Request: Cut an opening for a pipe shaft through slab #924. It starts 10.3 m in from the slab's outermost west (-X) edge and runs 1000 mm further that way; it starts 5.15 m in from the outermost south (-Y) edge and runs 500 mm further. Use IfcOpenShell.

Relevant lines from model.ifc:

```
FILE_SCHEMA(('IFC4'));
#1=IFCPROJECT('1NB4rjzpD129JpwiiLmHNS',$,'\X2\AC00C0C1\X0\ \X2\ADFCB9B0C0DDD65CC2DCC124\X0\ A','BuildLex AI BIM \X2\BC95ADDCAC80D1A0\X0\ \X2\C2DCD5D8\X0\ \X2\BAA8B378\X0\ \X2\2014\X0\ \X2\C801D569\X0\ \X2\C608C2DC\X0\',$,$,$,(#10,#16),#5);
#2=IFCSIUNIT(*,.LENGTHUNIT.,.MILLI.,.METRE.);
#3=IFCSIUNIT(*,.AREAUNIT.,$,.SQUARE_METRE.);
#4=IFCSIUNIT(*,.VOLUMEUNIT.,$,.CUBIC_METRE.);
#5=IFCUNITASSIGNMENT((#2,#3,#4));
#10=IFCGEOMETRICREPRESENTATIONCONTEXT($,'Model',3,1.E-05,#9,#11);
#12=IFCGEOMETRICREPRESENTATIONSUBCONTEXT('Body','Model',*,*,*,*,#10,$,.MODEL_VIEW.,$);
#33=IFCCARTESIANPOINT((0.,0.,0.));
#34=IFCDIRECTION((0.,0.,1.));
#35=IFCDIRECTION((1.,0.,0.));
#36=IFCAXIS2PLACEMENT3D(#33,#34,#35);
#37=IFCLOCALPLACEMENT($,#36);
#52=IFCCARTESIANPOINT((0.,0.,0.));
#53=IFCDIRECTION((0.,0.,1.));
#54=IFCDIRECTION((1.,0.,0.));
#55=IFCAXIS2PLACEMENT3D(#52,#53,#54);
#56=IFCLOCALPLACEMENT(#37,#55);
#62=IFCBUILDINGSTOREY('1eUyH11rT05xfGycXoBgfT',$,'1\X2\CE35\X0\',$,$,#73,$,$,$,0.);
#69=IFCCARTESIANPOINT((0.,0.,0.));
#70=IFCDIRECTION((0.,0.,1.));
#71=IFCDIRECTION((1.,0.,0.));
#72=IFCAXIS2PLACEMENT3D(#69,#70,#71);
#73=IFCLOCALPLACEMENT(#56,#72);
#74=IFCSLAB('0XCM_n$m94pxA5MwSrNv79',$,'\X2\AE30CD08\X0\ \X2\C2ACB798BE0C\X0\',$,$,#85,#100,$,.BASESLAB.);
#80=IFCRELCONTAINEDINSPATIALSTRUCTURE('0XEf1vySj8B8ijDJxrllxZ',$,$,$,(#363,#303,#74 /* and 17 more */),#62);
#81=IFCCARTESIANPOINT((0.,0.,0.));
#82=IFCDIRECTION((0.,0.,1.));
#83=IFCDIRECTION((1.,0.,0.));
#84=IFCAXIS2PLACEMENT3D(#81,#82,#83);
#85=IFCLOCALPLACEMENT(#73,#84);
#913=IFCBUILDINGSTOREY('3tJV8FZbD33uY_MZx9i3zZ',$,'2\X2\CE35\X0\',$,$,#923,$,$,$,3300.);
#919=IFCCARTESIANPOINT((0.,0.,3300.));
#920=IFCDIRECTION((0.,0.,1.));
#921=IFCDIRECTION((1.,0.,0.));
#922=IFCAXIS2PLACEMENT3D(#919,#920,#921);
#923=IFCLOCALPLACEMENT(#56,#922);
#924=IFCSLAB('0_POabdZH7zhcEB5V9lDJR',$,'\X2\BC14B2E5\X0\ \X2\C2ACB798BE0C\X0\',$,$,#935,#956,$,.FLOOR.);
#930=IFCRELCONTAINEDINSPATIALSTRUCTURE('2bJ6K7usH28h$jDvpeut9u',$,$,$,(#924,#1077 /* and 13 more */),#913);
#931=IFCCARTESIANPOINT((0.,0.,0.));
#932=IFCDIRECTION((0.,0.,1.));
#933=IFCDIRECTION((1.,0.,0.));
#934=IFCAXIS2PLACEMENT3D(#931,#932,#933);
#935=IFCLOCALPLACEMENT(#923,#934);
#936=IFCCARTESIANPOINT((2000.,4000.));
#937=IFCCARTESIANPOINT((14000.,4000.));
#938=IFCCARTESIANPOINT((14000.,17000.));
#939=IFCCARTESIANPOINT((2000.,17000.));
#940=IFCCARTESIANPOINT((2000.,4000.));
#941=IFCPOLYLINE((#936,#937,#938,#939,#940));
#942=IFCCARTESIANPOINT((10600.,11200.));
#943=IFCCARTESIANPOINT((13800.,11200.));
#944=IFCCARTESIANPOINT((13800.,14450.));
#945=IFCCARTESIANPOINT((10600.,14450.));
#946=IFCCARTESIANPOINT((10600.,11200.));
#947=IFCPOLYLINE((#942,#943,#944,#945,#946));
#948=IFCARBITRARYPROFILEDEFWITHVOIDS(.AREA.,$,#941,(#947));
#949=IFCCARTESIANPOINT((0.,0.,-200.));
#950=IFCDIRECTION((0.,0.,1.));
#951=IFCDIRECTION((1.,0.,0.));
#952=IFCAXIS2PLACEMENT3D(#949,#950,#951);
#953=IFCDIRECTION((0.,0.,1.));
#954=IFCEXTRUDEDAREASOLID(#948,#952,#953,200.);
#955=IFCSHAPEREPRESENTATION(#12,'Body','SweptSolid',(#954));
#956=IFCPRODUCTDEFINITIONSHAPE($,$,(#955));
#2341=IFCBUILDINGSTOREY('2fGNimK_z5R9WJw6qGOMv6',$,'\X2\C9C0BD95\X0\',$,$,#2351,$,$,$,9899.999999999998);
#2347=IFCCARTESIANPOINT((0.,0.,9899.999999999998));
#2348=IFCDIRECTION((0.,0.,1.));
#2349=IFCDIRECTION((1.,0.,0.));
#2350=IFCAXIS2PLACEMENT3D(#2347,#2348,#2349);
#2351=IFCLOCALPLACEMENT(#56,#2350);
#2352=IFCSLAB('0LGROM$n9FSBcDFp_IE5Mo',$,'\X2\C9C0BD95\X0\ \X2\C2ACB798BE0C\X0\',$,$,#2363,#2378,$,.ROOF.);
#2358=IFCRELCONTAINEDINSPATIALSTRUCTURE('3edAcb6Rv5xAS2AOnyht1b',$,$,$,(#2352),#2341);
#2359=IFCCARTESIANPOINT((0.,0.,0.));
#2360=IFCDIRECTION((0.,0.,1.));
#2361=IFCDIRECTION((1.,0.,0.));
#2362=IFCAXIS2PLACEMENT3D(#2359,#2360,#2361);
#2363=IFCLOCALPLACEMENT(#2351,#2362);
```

```python
import numpy as np
import ifcopenshell
import ifcopenshell.api.feature
import ifcopenshell.api.geometry
import ifcopenshell.api.root
import ifcopenshell.geom
import ifcopenshell.util.placement
import ifcopenshell.util.representation
import ifcopenshell.util.shape
import ifcopenshell.util.unit

model = ifcopenshell.open("model.ifc")
unit_scale = ifcopenshell.util.unit.calculate_unit_scale(model)
settings = ifcopenshell.geom.settings()


def volume(element):
    """Net volume in cubic metres, openings subtracted."""
    shape = ifcopenshell.geom.create_shape(settings, element)
    return ifcopenshell.util.shape.get_volume(shape.geometry)


slab = model.by_guid("0_POabdZH7zhcEB5V9lDJR")
before = volume(slab)

# Extent in the slab's own axes, in metres. The edges named are its -X and -Y sides.
slab_shape = ifcopenshell.geom.create_shape(settings, slab)
vertices = ifcopenshell.util.shape.get_vertices(slab_shape.geometry)
x_min, y_min, bottom = vertices.min(axis=0)
top = vertices[:, 2].max()

opening = ifcopenshell.api.root.create_entity(model, ifc_class="IfcOpeningElement", name="Pipe shaft opening", predefined_type="OPENING")
context = ifcopenshell.util.representation.get_context(model, "Model", "Body", "MODEL_VIEW")
width, depth = 1, 0.5
outline = [(0.0, 0.0), (width, 0.0), (width, depth), (0.0, depth), (0.0, 0.0)]
# Overshoot both faces by 50 mm so the cut is clean.
shape = ifcopenshell.api.geometry.add_slab_representation(
    model, context=context, depth=top - bottom + 0.1, polyline=outline
)
ifcopenshell.api.geometry.assign_representation(model, product=opening, representation=shape)

matrix = ifcopenshell.util.placement.get_local_placement(slab.ObjectPlacement)
matrix[:, 3] = matrix @ np.append(np.array([x_min + 10.3, y_min + 5.15, bottom - 0.05]) / unit_scale, 1.0)
ifcopenshell.api.geometry.edit_object_placement(model, product=opening, matrix=matrix, is_si=False)
ifcopenshell.api.feature.add_feature(model, feature=opening, element=slab)

after = volume(slab)

print(f"slab volume {before:.3f} -> {after:.3f} m3")

model.write("model_rev.ifc")
```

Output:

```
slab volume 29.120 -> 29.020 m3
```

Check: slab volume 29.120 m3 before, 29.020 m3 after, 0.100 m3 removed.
